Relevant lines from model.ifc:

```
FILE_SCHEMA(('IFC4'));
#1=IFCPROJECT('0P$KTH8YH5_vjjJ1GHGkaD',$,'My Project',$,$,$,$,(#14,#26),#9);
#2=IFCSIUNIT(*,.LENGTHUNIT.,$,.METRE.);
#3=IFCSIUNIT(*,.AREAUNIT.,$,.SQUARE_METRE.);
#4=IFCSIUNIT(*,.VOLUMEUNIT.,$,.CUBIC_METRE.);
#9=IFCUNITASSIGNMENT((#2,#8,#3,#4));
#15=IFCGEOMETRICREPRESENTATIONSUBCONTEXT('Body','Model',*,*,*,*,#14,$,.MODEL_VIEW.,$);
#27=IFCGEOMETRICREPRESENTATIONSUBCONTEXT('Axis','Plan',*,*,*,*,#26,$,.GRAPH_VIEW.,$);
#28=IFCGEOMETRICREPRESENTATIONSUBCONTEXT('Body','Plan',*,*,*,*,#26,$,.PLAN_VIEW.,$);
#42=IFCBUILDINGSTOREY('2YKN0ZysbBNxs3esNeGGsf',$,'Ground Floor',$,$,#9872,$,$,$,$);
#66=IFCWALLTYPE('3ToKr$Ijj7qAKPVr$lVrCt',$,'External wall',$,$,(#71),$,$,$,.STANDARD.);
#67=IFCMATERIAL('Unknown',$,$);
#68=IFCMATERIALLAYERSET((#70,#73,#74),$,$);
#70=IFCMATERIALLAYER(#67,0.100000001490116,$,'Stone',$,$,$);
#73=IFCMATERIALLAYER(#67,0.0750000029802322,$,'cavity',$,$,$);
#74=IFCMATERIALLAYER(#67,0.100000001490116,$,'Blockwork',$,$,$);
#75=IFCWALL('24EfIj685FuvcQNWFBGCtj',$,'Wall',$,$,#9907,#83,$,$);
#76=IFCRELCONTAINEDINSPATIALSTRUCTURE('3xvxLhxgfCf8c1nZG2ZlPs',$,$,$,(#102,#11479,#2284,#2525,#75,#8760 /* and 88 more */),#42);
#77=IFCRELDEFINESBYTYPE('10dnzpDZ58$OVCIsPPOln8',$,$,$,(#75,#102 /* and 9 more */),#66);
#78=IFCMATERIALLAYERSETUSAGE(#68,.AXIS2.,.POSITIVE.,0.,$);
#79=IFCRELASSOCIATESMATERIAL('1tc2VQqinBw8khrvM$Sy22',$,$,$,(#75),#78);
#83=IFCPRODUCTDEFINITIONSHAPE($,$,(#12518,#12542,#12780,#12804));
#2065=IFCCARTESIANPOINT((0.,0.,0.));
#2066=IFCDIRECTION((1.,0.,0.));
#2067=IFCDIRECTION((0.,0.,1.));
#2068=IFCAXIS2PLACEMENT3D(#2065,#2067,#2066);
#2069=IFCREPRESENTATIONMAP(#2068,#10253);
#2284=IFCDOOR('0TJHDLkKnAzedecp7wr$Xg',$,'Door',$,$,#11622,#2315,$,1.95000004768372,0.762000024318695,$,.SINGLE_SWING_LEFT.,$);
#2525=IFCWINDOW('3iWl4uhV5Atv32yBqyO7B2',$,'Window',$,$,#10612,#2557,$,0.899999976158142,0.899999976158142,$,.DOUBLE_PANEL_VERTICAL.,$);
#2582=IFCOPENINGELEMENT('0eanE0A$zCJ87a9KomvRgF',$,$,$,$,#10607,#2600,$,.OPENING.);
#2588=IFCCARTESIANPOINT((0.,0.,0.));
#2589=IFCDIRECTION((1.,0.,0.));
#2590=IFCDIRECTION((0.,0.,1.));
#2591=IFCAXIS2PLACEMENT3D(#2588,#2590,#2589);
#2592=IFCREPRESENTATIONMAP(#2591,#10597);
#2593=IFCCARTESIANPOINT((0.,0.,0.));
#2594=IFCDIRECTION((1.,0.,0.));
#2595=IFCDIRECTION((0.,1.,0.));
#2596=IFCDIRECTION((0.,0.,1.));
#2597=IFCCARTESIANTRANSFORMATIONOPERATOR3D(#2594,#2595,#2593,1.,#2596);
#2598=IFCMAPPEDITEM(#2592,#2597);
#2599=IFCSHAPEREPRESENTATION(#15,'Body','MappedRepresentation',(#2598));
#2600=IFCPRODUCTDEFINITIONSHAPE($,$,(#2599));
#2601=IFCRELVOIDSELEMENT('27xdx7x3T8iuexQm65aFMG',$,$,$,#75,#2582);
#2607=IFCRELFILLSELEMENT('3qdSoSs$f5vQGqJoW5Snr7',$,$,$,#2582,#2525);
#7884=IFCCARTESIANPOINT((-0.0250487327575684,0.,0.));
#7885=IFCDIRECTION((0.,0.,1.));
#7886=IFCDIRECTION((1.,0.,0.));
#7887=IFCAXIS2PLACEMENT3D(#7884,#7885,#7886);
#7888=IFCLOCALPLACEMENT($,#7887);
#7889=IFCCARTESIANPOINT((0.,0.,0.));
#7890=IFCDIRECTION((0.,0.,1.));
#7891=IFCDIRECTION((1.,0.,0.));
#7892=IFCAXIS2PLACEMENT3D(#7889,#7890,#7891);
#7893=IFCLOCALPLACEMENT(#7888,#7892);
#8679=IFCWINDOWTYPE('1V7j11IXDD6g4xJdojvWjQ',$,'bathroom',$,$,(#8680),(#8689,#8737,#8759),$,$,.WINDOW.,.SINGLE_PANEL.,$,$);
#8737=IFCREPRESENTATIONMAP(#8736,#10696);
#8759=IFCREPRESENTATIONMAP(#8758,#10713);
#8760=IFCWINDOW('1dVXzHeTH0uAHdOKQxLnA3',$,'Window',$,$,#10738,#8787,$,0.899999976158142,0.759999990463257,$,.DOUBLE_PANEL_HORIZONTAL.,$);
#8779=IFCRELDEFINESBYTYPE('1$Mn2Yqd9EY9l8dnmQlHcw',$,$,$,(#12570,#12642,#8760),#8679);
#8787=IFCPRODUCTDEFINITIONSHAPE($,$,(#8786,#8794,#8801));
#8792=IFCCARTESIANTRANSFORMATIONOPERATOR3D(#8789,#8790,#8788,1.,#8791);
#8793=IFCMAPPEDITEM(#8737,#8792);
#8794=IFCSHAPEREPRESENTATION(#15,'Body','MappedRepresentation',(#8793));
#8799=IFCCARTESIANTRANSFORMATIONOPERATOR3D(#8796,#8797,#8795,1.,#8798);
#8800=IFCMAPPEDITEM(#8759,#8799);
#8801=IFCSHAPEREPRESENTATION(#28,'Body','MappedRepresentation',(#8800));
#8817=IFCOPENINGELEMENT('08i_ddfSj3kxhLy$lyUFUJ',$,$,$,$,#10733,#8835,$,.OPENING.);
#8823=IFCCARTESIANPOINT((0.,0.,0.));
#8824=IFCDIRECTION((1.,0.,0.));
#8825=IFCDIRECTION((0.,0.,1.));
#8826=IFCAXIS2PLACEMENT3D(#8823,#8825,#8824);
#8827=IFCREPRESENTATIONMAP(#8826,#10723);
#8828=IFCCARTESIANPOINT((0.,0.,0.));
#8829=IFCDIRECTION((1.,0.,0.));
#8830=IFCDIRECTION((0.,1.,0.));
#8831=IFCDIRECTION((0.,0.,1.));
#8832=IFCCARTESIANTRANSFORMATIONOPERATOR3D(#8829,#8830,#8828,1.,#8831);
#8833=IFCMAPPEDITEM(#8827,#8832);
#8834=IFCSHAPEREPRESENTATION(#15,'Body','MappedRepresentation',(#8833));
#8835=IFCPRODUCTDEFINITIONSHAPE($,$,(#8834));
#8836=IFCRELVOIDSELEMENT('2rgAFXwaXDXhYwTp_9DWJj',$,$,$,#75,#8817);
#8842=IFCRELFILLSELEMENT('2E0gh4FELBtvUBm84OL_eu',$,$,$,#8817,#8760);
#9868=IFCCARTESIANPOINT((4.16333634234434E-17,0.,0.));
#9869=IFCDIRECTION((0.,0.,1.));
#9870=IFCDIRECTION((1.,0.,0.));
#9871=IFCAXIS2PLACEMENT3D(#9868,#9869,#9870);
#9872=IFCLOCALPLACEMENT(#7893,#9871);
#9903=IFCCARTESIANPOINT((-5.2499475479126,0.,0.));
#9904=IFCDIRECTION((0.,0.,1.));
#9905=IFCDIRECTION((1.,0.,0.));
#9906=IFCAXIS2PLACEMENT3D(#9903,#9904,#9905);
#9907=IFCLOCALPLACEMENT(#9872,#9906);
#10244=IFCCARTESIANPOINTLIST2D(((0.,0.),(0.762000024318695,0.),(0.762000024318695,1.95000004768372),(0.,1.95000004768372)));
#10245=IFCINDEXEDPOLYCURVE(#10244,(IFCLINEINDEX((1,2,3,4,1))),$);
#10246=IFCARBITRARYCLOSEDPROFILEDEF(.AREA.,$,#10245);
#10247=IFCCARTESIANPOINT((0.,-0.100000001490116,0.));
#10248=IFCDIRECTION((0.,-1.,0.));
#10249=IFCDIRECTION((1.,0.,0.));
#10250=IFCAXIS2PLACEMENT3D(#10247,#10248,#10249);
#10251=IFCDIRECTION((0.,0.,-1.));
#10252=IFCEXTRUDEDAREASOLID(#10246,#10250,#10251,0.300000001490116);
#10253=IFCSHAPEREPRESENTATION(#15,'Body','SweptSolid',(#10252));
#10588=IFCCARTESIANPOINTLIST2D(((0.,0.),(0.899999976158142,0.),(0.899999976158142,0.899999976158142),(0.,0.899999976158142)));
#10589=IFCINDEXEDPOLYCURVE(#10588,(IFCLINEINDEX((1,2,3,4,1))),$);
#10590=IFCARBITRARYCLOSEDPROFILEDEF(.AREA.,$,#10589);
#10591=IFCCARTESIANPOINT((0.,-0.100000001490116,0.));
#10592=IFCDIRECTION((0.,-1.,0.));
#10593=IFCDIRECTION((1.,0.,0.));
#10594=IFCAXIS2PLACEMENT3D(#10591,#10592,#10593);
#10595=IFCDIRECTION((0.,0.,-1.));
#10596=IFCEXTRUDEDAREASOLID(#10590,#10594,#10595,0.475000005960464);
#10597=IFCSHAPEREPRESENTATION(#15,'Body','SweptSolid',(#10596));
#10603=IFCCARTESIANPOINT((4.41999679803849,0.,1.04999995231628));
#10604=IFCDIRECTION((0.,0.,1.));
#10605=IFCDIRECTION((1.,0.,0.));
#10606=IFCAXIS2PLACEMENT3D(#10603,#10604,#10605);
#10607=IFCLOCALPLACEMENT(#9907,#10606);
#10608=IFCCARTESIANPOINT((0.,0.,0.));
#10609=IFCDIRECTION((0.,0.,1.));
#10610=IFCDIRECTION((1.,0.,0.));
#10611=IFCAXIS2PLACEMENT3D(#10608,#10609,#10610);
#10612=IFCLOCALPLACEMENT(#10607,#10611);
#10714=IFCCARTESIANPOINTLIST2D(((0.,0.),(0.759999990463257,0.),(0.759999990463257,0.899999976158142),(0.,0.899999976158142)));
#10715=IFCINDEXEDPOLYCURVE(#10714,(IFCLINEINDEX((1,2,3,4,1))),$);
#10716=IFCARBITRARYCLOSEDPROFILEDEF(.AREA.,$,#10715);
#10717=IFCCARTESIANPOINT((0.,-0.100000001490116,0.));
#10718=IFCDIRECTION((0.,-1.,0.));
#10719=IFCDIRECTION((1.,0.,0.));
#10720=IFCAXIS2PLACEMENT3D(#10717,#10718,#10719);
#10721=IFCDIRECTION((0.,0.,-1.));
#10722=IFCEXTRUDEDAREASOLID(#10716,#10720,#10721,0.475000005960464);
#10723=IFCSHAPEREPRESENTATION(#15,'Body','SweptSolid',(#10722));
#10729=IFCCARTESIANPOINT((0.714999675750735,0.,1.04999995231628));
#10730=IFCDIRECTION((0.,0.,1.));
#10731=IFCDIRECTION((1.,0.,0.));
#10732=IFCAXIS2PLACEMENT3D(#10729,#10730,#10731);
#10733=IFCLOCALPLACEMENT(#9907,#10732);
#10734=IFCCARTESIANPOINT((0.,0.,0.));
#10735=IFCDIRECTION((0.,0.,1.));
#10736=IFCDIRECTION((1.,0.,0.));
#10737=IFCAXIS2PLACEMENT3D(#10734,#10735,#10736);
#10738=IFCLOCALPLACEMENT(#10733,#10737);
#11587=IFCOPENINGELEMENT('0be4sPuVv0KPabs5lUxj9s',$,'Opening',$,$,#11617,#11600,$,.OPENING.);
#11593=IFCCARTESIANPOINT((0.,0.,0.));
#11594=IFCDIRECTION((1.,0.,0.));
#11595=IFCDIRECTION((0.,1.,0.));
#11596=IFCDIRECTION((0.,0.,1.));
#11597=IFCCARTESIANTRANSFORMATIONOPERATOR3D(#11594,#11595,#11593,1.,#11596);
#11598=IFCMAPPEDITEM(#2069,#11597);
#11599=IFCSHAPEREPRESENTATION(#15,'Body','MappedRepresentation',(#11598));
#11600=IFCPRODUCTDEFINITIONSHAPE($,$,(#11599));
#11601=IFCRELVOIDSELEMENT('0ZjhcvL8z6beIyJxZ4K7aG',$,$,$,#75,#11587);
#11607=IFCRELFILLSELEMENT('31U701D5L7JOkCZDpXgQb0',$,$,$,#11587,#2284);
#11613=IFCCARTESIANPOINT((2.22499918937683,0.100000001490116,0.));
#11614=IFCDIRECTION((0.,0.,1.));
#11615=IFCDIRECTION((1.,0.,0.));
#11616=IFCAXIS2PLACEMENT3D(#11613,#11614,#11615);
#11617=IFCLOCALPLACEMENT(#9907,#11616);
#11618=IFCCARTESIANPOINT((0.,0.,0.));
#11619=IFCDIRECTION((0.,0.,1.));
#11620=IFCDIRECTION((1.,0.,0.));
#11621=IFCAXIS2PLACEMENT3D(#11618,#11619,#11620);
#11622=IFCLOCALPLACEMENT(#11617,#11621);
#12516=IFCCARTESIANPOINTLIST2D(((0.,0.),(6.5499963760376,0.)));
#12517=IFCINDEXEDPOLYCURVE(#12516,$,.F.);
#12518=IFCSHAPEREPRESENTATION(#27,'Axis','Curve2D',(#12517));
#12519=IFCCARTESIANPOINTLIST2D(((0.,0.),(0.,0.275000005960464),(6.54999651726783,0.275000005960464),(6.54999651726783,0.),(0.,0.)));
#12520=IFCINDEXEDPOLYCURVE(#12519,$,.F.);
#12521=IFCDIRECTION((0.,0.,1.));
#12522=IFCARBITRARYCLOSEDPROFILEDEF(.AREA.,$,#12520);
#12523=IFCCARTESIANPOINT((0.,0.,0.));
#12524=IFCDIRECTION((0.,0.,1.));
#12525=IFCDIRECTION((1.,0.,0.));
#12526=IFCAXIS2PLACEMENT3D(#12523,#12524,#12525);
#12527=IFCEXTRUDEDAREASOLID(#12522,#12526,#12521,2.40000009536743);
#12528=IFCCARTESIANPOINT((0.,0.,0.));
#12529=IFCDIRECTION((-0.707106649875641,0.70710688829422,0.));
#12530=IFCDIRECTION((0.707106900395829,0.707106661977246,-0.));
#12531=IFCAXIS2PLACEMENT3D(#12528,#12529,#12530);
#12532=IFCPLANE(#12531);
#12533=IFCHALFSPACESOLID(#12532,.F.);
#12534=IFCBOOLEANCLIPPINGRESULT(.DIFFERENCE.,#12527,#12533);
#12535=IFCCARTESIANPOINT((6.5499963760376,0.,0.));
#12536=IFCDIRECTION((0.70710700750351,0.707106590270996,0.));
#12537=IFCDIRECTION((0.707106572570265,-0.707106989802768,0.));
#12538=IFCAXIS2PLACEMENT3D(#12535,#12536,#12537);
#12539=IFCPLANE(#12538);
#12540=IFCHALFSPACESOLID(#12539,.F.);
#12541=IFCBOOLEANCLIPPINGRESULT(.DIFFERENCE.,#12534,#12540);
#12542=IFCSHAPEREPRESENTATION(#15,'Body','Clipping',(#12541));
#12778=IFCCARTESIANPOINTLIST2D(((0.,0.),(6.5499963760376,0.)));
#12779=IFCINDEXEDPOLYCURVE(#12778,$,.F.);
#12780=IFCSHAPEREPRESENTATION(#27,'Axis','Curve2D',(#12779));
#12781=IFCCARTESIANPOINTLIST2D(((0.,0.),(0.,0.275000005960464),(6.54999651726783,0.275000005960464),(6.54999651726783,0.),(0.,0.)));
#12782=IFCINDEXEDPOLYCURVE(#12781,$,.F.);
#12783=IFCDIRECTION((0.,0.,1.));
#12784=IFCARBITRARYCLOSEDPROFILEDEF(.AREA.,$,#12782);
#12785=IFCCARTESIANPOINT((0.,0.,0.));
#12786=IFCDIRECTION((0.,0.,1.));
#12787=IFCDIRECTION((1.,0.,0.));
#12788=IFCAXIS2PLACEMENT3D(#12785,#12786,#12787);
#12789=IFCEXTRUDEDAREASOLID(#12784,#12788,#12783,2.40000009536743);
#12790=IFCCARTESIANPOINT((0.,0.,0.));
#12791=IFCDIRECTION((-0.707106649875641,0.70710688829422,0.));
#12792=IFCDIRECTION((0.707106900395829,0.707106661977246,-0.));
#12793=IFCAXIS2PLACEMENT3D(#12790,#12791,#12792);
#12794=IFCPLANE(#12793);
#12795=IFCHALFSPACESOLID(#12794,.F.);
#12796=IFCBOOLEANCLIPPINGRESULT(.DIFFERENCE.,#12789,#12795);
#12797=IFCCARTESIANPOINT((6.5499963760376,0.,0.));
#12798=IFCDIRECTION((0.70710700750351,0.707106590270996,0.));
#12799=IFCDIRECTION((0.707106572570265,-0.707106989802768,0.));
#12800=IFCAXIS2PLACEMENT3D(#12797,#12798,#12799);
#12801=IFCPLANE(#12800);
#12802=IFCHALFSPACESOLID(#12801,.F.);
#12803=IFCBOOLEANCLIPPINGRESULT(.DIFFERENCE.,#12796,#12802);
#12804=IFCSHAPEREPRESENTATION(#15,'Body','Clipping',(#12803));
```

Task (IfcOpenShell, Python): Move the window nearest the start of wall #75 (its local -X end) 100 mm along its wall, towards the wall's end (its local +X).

```python
import ifcopenshell
import ifcopenshell.api.geometry
import ifcopenshell.util.placement
import ifcopenshell.util.unit

model = ifcopenshell.open("model.ifc")
unit_scale = ifcopenshell.util.unit.calculate_unit_scale(model)

window = model.by_guid("1dVXzHeTH0uAHdOKQxLnA3")
opening = window.FillsVoids[0].RelatingOpeningElement
wall = opening.VoidsElements[0].RelatingBuildingElement

wall_matrix = ifcopenshell.util.placement.get_local_placement(wall.ObjectPlacement)
shift = wall_matrix[:3, 0] * 0.1 / unit_scale
before = ifcopenshell.util.placement.get_local_placement(window.ObjectPlacement)[:3, 3].copy()

# The window is placed relative to its opening, so it follows when the opening moves.
matrix = ifcopenshell.util.placement.get_local_placement(opening.ObjectPlacement)
matrix[:3, 3] += shift
ifcopenshell.api.geometry.edit_object_placement(
    model, product=opening, matrix=matrix, is_si=False, should_transform_children=True
)

after = ifcopenshell.util.placement.get_local_placement(window.ObjectPlacement)[:3, 3]
print("window moved by", (after - before).round(3) + 0.0)

model.write("model_edited.ifc")
```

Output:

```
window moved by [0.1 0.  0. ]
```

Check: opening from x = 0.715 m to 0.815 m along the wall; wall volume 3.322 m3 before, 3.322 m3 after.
